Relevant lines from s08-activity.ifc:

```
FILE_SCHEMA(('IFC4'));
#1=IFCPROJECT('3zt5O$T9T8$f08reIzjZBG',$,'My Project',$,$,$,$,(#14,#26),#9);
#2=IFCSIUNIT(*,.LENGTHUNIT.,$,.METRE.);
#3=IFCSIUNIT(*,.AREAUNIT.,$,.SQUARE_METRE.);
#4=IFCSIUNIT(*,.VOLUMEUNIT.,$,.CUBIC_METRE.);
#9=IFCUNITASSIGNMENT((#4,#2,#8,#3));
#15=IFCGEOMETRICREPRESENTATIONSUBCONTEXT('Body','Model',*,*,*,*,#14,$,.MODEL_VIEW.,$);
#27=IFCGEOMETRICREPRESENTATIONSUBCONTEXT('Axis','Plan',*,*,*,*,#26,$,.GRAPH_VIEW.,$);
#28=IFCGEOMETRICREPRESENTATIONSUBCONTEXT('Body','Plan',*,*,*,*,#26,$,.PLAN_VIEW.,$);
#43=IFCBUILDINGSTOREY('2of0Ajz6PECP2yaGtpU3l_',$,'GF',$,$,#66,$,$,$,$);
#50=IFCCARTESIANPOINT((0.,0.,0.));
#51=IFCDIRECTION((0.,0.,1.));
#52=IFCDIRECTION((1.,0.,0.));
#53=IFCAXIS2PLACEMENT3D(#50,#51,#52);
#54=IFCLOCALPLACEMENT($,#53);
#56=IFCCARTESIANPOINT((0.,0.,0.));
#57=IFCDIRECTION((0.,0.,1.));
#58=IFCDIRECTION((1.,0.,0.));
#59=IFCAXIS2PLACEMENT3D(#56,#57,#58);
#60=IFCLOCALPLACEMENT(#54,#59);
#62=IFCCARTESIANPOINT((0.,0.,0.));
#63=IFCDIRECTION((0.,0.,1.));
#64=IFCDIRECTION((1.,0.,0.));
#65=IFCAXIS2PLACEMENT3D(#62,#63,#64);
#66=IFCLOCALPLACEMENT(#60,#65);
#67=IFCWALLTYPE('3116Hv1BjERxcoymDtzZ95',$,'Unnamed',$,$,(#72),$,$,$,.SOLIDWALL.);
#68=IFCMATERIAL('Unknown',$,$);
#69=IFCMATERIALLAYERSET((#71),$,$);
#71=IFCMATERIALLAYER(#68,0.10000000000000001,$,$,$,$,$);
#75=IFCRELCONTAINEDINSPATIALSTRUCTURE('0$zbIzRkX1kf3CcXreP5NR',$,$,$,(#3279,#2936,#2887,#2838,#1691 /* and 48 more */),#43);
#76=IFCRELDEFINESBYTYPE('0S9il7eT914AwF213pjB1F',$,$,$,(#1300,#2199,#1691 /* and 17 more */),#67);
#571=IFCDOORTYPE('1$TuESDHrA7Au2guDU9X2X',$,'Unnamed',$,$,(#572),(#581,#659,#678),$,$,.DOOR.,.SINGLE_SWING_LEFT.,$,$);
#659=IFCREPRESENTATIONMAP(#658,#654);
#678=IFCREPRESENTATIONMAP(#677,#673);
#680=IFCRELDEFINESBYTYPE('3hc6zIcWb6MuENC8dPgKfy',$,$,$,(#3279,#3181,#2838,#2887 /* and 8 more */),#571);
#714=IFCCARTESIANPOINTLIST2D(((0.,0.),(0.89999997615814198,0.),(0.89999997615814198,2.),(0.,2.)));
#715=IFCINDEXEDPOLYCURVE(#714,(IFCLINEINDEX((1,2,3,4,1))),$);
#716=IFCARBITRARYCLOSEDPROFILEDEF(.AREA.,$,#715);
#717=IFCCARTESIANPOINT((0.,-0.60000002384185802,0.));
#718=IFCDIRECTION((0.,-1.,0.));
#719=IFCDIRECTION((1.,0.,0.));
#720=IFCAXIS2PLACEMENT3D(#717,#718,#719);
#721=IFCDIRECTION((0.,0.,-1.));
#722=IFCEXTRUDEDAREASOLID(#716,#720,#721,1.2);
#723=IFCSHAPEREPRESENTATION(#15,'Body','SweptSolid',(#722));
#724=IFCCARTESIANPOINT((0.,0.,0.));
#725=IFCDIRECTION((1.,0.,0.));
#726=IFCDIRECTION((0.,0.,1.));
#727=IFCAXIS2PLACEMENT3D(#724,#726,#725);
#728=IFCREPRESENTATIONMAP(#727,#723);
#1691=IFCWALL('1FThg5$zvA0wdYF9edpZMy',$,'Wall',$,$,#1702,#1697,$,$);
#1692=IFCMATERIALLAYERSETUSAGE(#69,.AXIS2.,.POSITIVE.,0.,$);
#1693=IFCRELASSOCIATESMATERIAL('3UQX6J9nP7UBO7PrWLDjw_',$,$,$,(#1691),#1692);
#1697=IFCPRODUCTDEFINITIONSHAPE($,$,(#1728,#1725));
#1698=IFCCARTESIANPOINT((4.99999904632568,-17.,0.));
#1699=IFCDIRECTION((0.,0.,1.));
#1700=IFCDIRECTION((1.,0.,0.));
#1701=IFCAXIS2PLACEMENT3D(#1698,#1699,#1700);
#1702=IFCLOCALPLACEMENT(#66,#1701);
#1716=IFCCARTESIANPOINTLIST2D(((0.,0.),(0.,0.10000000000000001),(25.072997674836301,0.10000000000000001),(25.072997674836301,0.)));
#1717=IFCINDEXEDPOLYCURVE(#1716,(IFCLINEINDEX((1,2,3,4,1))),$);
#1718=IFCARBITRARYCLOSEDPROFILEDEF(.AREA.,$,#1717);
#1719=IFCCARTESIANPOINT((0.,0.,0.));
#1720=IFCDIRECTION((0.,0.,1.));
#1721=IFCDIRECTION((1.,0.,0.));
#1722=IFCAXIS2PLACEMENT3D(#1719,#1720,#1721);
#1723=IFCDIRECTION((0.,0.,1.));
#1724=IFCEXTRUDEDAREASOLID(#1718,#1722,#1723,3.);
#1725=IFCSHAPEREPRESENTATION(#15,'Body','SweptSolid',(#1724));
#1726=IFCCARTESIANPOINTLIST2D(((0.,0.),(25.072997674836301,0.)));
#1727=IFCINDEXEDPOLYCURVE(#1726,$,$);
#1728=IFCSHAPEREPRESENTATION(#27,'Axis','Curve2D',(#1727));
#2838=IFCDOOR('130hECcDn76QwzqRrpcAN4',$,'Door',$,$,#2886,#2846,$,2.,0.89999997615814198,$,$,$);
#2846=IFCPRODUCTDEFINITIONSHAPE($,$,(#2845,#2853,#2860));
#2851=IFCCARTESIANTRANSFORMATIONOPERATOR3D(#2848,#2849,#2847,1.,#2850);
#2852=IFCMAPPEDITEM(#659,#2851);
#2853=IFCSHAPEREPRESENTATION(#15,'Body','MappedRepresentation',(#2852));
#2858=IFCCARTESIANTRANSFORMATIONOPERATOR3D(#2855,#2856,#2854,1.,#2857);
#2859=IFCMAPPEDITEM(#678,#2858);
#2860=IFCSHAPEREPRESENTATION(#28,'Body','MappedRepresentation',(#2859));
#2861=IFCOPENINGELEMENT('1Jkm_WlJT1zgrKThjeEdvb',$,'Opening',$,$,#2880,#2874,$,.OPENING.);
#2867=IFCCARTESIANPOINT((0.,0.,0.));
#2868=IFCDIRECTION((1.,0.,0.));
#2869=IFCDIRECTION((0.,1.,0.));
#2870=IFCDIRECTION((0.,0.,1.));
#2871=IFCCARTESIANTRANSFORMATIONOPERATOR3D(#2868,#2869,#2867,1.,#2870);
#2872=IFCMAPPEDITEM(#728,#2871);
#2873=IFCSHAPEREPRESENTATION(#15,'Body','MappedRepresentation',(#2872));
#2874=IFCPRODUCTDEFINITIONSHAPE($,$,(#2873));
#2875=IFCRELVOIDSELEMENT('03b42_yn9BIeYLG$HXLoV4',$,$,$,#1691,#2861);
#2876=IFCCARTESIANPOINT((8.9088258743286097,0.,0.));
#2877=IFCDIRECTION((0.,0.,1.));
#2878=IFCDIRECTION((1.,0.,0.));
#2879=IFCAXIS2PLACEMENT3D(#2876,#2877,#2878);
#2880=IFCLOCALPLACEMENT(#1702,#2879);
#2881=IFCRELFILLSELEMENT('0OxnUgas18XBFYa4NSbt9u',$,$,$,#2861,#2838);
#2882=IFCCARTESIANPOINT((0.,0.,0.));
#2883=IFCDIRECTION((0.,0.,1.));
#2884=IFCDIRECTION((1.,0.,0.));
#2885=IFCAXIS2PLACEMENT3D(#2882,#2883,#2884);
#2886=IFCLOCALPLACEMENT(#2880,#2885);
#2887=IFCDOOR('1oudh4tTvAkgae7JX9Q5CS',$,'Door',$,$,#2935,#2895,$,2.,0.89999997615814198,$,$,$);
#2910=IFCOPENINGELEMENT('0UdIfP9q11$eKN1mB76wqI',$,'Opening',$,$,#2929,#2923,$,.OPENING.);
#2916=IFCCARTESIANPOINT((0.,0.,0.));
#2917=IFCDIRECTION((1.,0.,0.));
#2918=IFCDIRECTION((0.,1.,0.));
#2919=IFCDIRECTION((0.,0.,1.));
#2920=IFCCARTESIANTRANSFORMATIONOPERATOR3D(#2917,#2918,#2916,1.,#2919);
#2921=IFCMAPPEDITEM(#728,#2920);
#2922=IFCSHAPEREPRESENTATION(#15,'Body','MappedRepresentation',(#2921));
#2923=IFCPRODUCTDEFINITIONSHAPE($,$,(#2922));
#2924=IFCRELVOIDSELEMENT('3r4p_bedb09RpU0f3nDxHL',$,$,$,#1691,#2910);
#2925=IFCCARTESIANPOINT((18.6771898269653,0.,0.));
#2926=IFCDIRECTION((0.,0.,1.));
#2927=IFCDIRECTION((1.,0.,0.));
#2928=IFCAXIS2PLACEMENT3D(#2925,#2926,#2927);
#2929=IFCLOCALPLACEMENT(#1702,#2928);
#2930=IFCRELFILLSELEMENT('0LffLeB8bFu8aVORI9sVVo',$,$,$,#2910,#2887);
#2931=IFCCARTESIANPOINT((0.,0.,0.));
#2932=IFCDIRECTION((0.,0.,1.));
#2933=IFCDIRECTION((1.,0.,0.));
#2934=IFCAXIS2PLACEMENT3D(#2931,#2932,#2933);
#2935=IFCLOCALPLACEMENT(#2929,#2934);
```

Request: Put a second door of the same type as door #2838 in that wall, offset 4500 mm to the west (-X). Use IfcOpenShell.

```python
import ifcopenshell
import ifcopenshell.api.feature
import ifcopenshell.api.geometry
import ifcopenshell.api.root
import ifcopenshell.geom
import ifcopenshell.util.element
import ifcopenshell.util.placement
import ifcopenshell.util.shape
import ifcopenshell.util.unit

model = ifcopenshell.open("s08-activity.ifc")
unit_scale = ifcopenshell.util.unit.calculate_unit_scale(model)
settings = ifcopenshell.geom.settings()


def volume(element):
    """Net volume in cubic metres, openings subtracted."""
    shape = ifcopenshell.geom.create_shape(settings, element)
    return ifcopenshell.util.shape.get_volume(shape.geometry)


door = model.by_guid("130hECcDn76QwzqRrpcAN4")
opening = door.FillsVoids[0].RelatingOpeningElement
wall = opening.VoidsElements[0].RelatingBuildingElement
before = volume(wall)
shift = ifcopenshell.util.placement.get_local_placement(wall.ObjectPlacement)[:3, 0] * -4.5 / unit_scale

# copy_class copies the void relationship, type, container and properties, but no geometry.
new_opening = ifcopenshell.api.root.copy_class(model, product=opening)
new_opening.Representation = ifcopenshell.util.element.copy_deep(
    model, opening.Representation, exclude=["IfcGeometricRepresentationContext", "IfcRepresentationMap"]
)
new_door = ifcopenshell.api.root.copy_class(model, product=door)
new_door.Representation = ifcopenshell.util.element.copy_deep(
    model, door.Representation, exclude=["IfcGeometricRepresentationContext", "IfcRepresentationMap"]
)
ifcopenshell.api.feature.add_filling(model, opening=new_opening, element=new_door)

for old, new in ((opening, new_opening), (door, new_door)):
    matrix = ifcopenshell.util.placement.get_local_placement(old.ObjectPlacement)
    matrix[:3, 3] += shift
    ifcopenshell.api.geometry.edit_object_placement(model, product=new, matrix=matrix, is_si=False)

after = volume(wall)

print(f"wall volume {before:.3f} -> {after:.3f} m3")

model.write("s08-activity_v2.ifc")
```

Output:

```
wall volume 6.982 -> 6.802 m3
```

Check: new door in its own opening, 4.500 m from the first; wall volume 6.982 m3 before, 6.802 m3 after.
